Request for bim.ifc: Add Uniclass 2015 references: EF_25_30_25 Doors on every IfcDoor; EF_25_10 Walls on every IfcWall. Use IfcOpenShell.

First a look at what the model holds.

```python
import ifcopenshell

model = ifcopenshell.open("bim.ifc")
print(model.schema)
print("classifications:", [c.Name for c in model.by_type("IfcClassification")])
for ifc_class in ("IfcDoor", "IfcRoof", "IfcStair", "IfcWall", "IfcWindow"):
    print(ifc_class, len(model.by_type(ifc_class)))
```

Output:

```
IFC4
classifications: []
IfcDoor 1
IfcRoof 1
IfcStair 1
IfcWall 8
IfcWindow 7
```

```python
import ifcopenshell
import ifcopenshell.api.classification

model = ifcopenshell.open("bim.ifc")

system = ifcopenshell.api.classification.add_classification(model, classification="Uniclass 2015")

codes = {
    "IfcDoor": ("EF_25_30_25", "Doors"),
    "IfcWall": ("EF_25_10", "Walls"),
}
for ifc_class, (code, name) in codes.items():
    products = model.by_type(ifc_class)
    ifcopenshell.api.classification.add_reference(
        model, products=products, classification=system, identification=code, name=name
    )
    print(code, len(products))

model.write("bim-out.ifc")
```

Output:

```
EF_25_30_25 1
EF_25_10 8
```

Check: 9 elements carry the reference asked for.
